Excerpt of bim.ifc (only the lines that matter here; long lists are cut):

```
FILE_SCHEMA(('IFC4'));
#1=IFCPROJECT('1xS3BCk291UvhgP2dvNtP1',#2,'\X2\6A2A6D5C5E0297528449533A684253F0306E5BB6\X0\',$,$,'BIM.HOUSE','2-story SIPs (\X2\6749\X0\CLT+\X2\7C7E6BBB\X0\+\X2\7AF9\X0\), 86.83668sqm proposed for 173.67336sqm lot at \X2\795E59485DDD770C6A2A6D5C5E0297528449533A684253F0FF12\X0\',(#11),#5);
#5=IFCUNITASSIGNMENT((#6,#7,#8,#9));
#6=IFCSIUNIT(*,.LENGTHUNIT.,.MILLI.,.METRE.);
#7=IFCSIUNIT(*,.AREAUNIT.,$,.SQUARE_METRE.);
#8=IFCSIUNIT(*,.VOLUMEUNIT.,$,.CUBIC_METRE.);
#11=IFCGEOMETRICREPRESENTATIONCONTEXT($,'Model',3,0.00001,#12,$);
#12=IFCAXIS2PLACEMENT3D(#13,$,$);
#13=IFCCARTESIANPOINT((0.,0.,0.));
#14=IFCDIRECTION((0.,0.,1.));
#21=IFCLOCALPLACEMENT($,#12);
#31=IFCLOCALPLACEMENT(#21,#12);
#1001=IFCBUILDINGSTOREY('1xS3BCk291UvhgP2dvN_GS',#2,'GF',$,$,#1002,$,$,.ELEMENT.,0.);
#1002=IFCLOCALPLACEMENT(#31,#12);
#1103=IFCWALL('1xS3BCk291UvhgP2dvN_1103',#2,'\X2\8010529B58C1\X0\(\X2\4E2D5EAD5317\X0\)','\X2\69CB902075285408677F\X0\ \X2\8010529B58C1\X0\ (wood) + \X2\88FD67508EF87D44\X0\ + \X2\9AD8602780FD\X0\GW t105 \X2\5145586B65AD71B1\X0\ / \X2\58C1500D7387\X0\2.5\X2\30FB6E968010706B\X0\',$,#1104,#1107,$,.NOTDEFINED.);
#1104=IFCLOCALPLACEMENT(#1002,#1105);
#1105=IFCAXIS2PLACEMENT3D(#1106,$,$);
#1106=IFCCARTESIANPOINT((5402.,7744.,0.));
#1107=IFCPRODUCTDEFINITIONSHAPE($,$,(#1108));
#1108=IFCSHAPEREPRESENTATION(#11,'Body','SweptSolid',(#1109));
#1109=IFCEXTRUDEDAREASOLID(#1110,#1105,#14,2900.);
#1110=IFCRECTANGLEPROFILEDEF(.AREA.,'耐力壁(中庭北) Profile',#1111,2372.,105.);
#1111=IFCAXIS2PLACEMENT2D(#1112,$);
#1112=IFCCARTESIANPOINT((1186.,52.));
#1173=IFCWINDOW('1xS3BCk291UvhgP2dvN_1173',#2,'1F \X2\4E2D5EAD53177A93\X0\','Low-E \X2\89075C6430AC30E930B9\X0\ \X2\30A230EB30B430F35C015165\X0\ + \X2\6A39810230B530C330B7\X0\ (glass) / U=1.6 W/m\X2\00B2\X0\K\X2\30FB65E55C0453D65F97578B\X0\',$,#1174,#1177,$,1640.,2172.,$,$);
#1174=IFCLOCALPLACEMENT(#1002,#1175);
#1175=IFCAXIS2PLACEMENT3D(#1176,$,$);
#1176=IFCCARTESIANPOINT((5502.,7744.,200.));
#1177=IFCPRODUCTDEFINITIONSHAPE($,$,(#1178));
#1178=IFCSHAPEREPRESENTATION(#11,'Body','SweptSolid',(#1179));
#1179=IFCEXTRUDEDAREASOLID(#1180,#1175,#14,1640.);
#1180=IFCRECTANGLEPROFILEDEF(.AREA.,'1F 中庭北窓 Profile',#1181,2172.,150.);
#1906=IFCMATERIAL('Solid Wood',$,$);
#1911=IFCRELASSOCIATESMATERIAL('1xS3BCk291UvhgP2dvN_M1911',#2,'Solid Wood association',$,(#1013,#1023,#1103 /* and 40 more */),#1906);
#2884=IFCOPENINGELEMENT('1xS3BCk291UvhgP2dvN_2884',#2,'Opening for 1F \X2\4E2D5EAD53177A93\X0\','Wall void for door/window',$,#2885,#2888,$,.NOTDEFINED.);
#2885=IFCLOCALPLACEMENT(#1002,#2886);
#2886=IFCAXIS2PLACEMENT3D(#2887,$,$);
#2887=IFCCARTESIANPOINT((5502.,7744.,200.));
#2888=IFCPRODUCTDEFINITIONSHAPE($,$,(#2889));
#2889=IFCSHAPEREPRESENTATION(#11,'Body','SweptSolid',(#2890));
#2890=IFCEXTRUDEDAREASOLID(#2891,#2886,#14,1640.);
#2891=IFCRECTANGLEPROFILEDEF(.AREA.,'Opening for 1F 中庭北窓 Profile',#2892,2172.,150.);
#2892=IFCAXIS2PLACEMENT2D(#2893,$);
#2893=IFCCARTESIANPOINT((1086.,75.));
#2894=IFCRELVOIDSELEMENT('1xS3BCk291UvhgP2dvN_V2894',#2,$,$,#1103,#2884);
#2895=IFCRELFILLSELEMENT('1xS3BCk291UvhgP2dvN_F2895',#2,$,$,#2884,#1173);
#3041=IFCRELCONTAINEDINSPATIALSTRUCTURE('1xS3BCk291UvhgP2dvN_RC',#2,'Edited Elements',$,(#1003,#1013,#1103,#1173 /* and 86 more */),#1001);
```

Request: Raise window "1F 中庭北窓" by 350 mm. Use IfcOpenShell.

```python
import numpy as np
import ifcopenshell
import ifcopenshell.api.geometry
import ifcopenshell.util.placement
import ifcopenshell.util.unit

model = ifcopenshell.open("bim.ifc")
unit_scale = ifcopenshell.util.unit.calculate_unit_scale(model)

window = model.by_id(1173)
opening = window.FillsVoids[0].RelatingOpeningElement
dz = 0.35 / unit_scale

shift = np.array([0.0, 0.0, dz])
# The window is not placed relative to its opening, so move both.
for product in (opening, window):
    matrix = ifcopenshell.util.placement.get_local_placement(product.ObjectPlacement)
    matrix[:3, 3] += shift
    ifcopenshell.api.geometry.edit_object_placement(model, product=product, matrix=matrix, is_si=False)

print(f"moved by {dz * unit_scale:+.3f} m")

model.write("bim_v2.ifc")
```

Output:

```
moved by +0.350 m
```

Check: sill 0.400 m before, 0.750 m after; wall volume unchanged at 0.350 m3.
